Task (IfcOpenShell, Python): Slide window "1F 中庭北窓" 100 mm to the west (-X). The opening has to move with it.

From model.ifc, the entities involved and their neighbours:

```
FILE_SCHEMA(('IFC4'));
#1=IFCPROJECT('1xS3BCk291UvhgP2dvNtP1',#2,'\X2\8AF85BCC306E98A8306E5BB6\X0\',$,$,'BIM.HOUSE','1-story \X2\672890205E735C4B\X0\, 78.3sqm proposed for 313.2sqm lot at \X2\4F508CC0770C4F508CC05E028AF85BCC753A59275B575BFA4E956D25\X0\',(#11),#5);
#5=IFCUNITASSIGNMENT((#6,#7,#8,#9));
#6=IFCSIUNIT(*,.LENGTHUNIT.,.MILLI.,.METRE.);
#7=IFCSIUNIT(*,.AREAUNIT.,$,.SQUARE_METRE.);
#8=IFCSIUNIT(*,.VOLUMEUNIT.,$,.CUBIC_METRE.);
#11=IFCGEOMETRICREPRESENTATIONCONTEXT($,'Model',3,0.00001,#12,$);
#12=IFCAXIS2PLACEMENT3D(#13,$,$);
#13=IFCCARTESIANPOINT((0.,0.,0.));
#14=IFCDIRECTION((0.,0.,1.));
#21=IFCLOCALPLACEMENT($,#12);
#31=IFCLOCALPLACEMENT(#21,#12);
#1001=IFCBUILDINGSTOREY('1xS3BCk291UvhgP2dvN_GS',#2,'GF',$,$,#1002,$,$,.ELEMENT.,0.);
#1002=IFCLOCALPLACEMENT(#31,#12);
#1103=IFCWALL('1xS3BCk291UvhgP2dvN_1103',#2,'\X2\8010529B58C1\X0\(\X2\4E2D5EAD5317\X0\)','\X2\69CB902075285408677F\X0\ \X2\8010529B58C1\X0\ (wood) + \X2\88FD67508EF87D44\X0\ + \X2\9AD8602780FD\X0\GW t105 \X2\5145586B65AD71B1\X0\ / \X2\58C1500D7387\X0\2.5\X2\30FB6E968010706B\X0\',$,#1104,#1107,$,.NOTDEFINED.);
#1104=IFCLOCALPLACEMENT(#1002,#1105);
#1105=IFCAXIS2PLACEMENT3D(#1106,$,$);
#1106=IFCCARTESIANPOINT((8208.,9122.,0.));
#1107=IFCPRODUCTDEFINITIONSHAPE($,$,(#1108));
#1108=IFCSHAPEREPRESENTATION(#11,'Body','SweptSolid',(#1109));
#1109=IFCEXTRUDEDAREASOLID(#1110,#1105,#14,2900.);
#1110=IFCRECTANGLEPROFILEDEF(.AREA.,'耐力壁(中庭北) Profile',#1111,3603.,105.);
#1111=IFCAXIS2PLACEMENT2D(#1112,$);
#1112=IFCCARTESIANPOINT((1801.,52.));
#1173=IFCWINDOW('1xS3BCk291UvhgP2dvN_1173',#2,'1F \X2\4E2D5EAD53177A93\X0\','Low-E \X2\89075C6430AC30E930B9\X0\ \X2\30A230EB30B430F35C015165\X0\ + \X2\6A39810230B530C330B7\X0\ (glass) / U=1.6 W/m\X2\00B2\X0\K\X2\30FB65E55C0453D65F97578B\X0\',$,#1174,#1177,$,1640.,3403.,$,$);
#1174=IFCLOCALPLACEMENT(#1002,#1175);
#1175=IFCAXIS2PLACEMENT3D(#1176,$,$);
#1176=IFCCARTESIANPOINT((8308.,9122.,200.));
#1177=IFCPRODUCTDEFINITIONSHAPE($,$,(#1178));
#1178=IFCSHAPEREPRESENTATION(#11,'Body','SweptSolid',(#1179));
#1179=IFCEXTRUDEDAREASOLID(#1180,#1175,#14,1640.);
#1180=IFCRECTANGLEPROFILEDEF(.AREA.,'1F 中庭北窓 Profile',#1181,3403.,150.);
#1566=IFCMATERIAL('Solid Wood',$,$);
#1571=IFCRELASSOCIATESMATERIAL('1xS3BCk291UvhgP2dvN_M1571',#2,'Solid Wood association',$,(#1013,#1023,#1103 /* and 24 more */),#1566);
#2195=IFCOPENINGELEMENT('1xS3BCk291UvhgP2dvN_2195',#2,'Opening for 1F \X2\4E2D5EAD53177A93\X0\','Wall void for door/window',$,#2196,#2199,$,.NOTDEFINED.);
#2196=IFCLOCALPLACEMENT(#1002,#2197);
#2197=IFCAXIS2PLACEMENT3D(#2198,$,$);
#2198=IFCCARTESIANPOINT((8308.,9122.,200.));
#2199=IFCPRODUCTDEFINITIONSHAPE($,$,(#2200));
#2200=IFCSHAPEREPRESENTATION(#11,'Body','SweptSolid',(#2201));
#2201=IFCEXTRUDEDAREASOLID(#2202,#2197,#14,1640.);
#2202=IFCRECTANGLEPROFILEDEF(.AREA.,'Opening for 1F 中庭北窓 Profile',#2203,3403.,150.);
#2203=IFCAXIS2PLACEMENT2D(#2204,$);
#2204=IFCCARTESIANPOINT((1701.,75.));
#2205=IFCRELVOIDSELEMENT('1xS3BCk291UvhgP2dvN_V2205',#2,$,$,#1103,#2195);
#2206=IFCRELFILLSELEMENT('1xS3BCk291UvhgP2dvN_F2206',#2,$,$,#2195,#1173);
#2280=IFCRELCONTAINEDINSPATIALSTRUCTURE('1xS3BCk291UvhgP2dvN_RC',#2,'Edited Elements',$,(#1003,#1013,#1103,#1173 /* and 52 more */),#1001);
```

```python
import ifcopenshell
import ifcopenshell.api.geometry
import ifcopenshell.util.placement
import ifcopenshell.util.unit

model = ifcopenshell.open("model.ifc")
unit_scale = ifcopenshell.util.unit.calculate_unit_scale(model)

window = model.by_id(1173)
opening = window.FillsVoids[0].RelatingOpeningElement
wall = opening.VoidsElements[0].RelatingBuildingElement

wall_matrix = ifcopenshell.util.placement.get_local_placement(wall.ObjectPlacement)
shift = wall_matrix[:3, 0] * -0.1 / unit_scale
before = ifcopenshell.util.placement.get_local_placement(window.ObjectPlacement)[:3, 3].copy()

# The window is not placed relative to its opening, so move both.
for product in (opening, window):
    matrix = ifcopenshell.util.placement.get_local_placement(product.ObjectPlacement)
    matrix[:3, 3] += shift
    ifcopenshell.api.geometry.edit_object_placement(model, product=product, matrix=matrix, is_si=False)

after = ifcopenshell.util.placement.get_local_placement(window.ObjectPlacement)[:3, 3]
print("window moved by", (after - before).round(3) + 0.0)

model.write("model_edited.ifc")
```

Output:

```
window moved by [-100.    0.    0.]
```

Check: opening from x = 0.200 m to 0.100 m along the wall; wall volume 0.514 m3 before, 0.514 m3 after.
